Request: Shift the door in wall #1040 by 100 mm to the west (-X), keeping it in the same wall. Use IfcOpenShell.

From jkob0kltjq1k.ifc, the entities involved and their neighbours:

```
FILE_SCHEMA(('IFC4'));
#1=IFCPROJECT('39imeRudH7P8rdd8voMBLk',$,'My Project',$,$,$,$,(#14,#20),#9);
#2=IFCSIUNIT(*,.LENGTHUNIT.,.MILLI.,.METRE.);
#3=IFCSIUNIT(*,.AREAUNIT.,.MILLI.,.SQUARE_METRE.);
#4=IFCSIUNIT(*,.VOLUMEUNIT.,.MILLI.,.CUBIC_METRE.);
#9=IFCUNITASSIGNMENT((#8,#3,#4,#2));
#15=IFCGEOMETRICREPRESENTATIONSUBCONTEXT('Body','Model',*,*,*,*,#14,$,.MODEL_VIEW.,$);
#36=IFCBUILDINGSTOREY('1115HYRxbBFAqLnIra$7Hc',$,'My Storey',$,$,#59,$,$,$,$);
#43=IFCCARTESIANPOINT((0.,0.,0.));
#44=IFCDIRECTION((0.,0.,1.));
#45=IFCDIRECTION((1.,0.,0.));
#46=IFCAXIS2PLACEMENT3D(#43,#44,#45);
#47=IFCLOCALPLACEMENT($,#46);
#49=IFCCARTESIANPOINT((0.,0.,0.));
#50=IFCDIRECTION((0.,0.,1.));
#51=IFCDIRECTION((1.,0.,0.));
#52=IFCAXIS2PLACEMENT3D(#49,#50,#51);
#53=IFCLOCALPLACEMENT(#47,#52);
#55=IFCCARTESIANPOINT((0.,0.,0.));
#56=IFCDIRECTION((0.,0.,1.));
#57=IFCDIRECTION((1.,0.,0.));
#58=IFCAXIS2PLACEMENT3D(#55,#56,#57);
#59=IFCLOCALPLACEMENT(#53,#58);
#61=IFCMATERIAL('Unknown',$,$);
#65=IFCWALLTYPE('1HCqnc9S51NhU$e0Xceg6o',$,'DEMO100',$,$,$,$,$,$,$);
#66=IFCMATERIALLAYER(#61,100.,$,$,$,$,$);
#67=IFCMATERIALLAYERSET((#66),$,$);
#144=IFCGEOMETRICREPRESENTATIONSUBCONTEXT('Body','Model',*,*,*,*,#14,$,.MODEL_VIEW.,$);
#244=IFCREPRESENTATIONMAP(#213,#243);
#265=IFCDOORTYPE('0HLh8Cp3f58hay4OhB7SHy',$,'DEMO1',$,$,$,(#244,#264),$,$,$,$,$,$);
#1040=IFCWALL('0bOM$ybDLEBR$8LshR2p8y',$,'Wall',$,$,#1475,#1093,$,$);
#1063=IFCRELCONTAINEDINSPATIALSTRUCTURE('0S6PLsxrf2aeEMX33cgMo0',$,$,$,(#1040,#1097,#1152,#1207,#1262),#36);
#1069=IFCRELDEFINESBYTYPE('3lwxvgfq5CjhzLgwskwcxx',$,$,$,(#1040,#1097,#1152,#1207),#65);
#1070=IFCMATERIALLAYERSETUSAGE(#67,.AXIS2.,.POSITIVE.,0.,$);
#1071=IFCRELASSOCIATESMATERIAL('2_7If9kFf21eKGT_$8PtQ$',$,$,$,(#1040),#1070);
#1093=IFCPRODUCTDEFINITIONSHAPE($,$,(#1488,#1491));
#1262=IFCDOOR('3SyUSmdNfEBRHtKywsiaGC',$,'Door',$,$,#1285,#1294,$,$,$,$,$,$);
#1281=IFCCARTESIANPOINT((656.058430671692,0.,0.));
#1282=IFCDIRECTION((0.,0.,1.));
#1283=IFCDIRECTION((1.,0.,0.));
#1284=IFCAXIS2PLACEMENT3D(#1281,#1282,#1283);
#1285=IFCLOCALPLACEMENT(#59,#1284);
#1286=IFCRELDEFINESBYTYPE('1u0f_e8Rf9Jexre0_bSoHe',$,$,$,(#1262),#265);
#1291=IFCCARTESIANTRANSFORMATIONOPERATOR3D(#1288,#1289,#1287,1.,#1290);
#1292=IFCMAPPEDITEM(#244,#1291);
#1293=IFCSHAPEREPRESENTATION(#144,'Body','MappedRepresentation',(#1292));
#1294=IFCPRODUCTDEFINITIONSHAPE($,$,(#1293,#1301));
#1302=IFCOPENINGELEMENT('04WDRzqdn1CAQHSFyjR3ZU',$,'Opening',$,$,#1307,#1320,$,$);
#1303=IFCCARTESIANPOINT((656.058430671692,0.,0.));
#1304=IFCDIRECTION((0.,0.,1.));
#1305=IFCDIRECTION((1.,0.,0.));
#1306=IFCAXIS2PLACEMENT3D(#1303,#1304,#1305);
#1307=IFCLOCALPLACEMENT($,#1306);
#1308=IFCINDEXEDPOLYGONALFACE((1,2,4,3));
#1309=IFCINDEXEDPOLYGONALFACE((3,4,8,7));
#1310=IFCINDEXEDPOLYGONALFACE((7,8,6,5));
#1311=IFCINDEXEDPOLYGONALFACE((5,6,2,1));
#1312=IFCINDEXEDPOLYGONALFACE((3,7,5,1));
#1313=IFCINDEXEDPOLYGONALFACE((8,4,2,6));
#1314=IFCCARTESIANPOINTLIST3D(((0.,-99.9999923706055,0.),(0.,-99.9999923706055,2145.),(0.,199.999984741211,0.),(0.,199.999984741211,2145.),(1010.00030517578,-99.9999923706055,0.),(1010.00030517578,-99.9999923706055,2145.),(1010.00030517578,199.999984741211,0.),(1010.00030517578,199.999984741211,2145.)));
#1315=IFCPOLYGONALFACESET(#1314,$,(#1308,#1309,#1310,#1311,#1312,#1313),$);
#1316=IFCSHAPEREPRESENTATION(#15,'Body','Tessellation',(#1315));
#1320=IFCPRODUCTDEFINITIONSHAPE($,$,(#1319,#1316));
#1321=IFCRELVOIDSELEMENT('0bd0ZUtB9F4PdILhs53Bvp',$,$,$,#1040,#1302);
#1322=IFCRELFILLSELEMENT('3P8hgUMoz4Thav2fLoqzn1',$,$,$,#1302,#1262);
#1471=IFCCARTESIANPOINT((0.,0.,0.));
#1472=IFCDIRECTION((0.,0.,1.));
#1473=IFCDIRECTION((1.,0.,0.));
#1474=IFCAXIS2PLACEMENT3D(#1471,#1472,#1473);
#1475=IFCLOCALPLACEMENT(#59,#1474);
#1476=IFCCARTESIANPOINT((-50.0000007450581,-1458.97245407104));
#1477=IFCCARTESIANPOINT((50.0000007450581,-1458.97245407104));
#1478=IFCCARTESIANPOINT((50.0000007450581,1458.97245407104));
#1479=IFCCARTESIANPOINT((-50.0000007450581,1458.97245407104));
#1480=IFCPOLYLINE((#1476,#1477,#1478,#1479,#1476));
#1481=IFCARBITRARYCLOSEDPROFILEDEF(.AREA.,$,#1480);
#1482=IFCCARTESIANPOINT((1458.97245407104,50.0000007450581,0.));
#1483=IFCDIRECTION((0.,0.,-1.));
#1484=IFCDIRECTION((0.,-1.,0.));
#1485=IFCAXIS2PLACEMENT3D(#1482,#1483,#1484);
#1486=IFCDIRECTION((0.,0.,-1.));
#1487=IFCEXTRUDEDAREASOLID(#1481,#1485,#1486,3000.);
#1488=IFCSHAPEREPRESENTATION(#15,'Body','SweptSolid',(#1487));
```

```python
import ifcopenshell
import ifcopenshell.api.geometry
import ifcopenshell.util.placement

model = ifcopenshell.open("jkob0kltjq1k.ifc")

door = model.by_guid("3SyUSmdNfEBRHtKywsiaGC")
opening = door.FillsVoids[0].RelatingOpeningElement
wall = opening.VoidsElements[0].RelatingBuildingElement

wall_matrix = ifcopenshell.util.placement.get_local_placement(wall.ObjectPlacement)
shift = wall_matrix[:3, 0] * -100.0
before = ifcopenshell.util.placement.get_local_placement(door.ObjectPlacement)[:3, 3].copy()

# The door is not placed relative to its opening, so move both.
for product in (opening, door):
    matrix = ifcopenshell.util.placement.get_local_placement(product.ObjectPlacement)
    matrix[:3, 3] += shift
    ifcopenshell.api.geometry.edit_object_placement(model, product=product, matrix=matrix, is_si=False)

after = ifcopenshell.util.placement.get_local_placement(door.ObjectPlacement)[:3, 3]
print("door moved by", (after - before).round(3) + 0.0)

model.write("jkob0kltjq1k-out.ifc")
```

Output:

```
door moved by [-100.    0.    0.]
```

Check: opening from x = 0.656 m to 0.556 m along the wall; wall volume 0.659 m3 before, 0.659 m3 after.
